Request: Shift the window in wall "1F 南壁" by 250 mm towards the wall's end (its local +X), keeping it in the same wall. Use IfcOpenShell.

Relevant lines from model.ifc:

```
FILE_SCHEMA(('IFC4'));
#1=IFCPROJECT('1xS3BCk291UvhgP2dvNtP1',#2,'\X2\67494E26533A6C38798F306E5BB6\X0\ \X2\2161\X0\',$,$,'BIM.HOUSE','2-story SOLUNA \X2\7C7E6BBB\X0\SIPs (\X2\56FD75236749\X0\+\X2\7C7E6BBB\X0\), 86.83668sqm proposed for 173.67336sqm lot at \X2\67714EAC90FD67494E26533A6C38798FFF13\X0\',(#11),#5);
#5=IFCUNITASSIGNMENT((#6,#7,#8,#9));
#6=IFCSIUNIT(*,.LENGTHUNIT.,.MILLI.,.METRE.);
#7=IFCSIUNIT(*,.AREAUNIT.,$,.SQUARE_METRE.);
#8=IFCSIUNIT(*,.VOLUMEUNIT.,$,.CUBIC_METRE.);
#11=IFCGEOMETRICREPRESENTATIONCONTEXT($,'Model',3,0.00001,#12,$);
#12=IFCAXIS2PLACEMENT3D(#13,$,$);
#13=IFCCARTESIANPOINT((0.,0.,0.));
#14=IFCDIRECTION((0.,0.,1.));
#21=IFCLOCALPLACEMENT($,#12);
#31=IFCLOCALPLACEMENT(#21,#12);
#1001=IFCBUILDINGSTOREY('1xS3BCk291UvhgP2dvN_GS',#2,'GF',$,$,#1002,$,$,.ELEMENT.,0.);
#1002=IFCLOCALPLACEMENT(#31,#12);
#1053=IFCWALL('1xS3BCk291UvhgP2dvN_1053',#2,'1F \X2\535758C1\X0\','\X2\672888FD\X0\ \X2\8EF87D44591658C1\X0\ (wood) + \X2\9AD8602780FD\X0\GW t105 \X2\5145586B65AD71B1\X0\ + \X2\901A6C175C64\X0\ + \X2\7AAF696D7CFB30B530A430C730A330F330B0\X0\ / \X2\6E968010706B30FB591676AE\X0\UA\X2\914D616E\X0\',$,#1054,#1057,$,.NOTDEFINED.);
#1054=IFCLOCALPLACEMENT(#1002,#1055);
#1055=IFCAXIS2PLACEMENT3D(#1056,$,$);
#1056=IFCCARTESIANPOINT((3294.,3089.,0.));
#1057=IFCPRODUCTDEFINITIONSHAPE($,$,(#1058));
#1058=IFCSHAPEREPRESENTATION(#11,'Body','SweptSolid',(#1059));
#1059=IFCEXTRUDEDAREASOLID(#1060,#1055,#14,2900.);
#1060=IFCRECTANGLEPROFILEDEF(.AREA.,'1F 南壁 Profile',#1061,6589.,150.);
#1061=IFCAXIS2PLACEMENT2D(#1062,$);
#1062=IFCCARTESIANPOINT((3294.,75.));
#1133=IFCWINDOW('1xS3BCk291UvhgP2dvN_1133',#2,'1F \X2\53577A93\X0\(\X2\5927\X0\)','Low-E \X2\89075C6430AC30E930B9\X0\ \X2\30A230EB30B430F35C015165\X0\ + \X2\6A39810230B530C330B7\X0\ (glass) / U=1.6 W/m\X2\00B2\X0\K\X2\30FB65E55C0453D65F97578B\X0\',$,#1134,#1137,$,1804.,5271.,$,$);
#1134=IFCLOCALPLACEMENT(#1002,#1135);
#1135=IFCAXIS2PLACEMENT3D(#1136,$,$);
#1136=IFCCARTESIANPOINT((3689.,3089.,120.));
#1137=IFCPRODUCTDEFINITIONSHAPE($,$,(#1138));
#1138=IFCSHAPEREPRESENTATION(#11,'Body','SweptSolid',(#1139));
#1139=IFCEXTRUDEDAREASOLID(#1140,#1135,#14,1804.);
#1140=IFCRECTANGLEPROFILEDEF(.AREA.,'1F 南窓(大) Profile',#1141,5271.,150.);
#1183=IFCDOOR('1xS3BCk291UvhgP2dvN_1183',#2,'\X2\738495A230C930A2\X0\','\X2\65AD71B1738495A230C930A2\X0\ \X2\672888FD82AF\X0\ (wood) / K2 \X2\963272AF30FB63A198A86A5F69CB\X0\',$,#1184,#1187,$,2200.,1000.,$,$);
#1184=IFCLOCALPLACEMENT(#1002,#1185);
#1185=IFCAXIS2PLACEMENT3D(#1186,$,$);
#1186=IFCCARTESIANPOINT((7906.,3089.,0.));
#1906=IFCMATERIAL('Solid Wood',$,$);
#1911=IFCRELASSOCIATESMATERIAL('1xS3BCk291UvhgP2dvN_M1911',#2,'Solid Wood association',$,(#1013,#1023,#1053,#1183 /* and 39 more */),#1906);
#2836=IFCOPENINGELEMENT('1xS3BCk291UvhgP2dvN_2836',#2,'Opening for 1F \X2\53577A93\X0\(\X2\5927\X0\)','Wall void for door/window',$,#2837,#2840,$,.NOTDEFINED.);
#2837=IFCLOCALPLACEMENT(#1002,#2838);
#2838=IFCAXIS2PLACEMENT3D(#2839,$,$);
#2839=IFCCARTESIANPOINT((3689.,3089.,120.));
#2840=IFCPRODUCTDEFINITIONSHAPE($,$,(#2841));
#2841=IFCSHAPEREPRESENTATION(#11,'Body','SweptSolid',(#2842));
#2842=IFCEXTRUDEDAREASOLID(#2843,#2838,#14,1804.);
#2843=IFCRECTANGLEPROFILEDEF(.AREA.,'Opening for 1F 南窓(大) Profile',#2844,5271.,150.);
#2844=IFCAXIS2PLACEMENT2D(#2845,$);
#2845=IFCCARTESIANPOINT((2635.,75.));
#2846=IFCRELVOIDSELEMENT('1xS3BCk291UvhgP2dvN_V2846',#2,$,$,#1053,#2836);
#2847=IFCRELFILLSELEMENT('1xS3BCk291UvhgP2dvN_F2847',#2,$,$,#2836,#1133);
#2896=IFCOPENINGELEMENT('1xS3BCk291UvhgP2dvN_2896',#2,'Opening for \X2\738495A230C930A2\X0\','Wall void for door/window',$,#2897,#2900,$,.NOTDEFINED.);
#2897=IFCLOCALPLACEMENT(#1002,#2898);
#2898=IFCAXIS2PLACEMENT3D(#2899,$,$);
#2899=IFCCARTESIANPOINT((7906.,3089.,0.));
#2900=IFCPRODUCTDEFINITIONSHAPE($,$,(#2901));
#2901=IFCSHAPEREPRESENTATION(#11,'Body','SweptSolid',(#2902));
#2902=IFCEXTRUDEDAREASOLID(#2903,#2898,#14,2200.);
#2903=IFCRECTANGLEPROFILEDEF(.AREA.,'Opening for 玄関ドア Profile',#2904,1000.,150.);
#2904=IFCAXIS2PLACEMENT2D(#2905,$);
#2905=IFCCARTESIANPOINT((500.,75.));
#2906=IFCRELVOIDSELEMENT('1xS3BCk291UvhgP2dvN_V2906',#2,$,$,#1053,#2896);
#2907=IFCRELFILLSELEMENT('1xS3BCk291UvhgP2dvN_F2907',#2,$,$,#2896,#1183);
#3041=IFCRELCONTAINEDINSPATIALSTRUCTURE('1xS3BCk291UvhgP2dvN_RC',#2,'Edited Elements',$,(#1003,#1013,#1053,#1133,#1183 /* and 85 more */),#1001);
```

```python
import ifcopenshell
import ifcopenshell.api.geometry
import ifcopenshell.util.placement

model = ifcopenshell.open("model.ifc")

window = model.by_id(1133)
opening = window.FillsVoids[0].RelatingOpeningElement
wall = opening.VoidsElements[0].RelatingBuildingElement

wall_matrix = ifcopenshell.util.placement.get_local_placement(wall.ObjectPlacement)
shift = wall_matrix[:3, 0] * 250.0
before = ifcopenshell.util.placement.get_local_placement(window.ObjectPlacement)[:3, 3].copy()

# The window is not placed relative to its opening, so move both.
for product in (opening, window):
    matrix = ifcopenshell.util.placement.get_local_placement(product.ObjectPlacement)
    matrix[:3, 3] += shift
    ifcopenshell.api.geometry.edit_object_placement(model, product=product, matrix=matrix, is_si=False)

after = ifcopenshell.util.placement.get_local_placement(window.ObjectPlacement)[:3, 3]
print("window moved by", (after - before).round(3) + 0.0)

model.write("model_v2.ifc")
```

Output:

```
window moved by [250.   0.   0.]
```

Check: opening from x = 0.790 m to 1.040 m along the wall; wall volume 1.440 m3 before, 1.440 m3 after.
